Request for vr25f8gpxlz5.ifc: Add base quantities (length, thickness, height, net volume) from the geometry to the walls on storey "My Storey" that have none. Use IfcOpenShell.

First a look at what the model holds.

```python
import ifcopenshell
import ifcopenshell.util.element
import ifcopenshell.util.unit

model = ifcopenshell.open("vr25f8gpxlz5.ifc")
print(model.schema)
for unit_type in ("LENGTHUNIT", "AREAUNIT", "VOLUMEUNIT"):
    print(unit_type, ifcopenshell.util.unit.calculate_unit_scale(model, unit_type))
storey = next(s for s in model.by_type("IfcBuildingStorey") if s.Name == "My Storey")
walls = [e for e in ifcopenshell.util.element.get_decomposition(storey) if e.is_a("IfcWall")]
for e in sorted(walls, key=lambda e: e.id()):
    print(e.id(), e.is_a(), e.Name, list(ifcopenshell.util.element.get_psets(e, qtos_only=True)), sep=" | ")
```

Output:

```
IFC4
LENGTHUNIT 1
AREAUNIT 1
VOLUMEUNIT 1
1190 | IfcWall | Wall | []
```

```python
import ifcopenshell
import ifcopenshell.api.pset
import ifcopenshell.geom
import ifcopenshell.util.element
import ifcopenshell.util.shape
import ifcopenshell.util.unit

model = ifcopenshell.open("vr25f8gpxlz5.ifc")
unit_scale = ifcopenshell.util.unit.calculate_unit_scale(model)
volume_scale = ifcopenshell.util.unit.calculate_unit_scale(model, "VOLUMEUNIT")
settings = ifcopenshell.geom.settings()

storey = next(s for s in model.by_type("IfcBuildingStorey") if s.Name == "My Storey")
walls = [e for e in ifcopenshell.util.element.get_decomposition(storey) if e.is_a("IfcWall")]

for e in sorted(walls, key=lambda e: e.id()):
    if ifcopenshell.util.element.get_psets(e, qtos_only=True, should_inherit=False):
        continue
    # Geometry comes back in metres, in the element's own axes.
    shape = ifcopenshell.geom.create_shape(settings, e)
    values = {
        "Length": ifcopenshell.util.shape.get_x(shape.geometry) / unit_scale,
        "Width": ifcopenshell.util.shape.get_y(shape.geometry) / unit_scale,
        "Height": ifcopenshell.util.shape.get_z(shape.geometry) / unit_scale,
        "NetVolume": ifcopenshell.util.shape.get_volume(shape.geometry) / volume_scale,
    }
    qto = ifcopenshell.api.pset.add_qto(model, product=e, name="Qto_WallBaseQuantities")
    ifcopenshell.api.pset.edit_qto(model, qto=qto, properties=values)
    print(e.id(), {k: round(v, 3) for k, v in values.items()})

model.write("vr25f8gpxlz5_v2.ifc")
```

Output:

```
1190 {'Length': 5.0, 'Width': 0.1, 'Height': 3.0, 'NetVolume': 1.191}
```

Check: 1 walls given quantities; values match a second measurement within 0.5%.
